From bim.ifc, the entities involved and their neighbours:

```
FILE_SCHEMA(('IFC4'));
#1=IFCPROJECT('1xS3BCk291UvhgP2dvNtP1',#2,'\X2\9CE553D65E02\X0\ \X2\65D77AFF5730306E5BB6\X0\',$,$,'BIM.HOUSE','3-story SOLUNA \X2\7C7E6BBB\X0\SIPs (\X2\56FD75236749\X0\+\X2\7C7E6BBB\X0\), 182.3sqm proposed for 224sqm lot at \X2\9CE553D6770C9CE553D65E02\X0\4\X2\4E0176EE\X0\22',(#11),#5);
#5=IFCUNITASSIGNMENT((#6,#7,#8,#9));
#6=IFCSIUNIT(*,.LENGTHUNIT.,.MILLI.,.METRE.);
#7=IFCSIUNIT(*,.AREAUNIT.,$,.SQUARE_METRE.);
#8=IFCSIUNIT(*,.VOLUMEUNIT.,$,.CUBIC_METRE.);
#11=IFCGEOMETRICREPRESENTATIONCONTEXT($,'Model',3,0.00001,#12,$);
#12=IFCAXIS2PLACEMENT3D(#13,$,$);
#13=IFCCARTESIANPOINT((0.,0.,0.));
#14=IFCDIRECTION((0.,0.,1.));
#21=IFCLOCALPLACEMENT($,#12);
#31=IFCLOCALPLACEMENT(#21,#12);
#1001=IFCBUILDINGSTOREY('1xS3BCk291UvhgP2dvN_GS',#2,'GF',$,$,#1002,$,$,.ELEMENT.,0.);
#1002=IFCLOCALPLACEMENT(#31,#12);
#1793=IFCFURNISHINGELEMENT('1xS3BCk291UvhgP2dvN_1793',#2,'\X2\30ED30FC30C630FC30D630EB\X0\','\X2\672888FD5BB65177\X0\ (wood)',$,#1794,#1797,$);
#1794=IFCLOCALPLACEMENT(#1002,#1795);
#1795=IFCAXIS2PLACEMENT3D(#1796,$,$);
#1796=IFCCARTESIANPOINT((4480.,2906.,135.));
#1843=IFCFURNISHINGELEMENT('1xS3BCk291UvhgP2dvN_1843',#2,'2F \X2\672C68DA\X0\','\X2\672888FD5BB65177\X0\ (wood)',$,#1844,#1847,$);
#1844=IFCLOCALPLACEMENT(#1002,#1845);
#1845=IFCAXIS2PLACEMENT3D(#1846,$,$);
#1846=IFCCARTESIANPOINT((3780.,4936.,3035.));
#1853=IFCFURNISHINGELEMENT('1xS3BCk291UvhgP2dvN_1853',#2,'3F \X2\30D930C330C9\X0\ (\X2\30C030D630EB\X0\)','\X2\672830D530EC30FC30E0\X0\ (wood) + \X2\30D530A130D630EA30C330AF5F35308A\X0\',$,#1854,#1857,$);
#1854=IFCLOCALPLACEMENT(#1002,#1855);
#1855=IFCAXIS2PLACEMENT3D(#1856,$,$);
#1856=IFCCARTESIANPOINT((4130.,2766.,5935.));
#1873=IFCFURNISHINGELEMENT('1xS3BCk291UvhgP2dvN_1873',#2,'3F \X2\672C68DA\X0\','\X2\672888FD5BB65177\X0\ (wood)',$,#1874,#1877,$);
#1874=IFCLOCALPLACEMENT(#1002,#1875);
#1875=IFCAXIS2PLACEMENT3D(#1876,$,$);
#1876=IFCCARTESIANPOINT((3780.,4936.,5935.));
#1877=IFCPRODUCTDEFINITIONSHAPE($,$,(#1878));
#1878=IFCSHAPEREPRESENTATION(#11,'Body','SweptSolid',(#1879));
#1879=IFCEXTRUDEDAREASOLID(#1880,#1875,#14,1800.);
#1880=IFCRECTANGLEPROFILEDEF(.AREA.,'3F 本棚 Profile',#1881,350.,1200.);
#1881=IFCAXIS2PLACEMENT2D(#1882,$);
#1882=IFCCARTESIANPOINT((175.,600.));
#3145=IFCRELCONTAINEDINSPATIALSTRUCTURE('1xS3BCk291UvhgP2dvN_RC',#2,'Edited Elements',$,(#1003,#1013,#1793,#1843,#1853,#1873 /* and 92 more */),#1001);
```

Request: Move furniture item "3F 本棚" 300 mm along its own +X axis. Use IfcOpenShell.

```python
import ifcopenshell
import ifcopenshell.api.geometry
import ifcopenshell.util.placement

model = ifcopenshell.open("bim.ifc")

item = model.by_id(1873)
matrix = ifcopenshell.util.placement.get_local_placement(item.ObjectPlacement)
matrix[:3, 3] += matrix[:3, 0] * 300.0
ifcopenshell.api.geometry.edit_object_placement(model, product=item, matrix=matrix, is_si=False)

print(ifcopenshell.util.placement.get_local_placement(item.ObjectPlacement).round(3) + 0.0)

model.write("bim_rev.ifc")
```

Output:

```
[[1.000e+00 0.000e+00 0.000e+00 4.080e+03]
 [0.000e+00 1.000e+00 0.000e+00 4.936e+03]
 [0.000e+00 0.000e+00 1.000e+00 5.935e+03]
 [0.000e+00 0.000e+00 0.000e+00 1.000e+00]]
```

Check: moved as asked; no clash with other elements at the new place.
